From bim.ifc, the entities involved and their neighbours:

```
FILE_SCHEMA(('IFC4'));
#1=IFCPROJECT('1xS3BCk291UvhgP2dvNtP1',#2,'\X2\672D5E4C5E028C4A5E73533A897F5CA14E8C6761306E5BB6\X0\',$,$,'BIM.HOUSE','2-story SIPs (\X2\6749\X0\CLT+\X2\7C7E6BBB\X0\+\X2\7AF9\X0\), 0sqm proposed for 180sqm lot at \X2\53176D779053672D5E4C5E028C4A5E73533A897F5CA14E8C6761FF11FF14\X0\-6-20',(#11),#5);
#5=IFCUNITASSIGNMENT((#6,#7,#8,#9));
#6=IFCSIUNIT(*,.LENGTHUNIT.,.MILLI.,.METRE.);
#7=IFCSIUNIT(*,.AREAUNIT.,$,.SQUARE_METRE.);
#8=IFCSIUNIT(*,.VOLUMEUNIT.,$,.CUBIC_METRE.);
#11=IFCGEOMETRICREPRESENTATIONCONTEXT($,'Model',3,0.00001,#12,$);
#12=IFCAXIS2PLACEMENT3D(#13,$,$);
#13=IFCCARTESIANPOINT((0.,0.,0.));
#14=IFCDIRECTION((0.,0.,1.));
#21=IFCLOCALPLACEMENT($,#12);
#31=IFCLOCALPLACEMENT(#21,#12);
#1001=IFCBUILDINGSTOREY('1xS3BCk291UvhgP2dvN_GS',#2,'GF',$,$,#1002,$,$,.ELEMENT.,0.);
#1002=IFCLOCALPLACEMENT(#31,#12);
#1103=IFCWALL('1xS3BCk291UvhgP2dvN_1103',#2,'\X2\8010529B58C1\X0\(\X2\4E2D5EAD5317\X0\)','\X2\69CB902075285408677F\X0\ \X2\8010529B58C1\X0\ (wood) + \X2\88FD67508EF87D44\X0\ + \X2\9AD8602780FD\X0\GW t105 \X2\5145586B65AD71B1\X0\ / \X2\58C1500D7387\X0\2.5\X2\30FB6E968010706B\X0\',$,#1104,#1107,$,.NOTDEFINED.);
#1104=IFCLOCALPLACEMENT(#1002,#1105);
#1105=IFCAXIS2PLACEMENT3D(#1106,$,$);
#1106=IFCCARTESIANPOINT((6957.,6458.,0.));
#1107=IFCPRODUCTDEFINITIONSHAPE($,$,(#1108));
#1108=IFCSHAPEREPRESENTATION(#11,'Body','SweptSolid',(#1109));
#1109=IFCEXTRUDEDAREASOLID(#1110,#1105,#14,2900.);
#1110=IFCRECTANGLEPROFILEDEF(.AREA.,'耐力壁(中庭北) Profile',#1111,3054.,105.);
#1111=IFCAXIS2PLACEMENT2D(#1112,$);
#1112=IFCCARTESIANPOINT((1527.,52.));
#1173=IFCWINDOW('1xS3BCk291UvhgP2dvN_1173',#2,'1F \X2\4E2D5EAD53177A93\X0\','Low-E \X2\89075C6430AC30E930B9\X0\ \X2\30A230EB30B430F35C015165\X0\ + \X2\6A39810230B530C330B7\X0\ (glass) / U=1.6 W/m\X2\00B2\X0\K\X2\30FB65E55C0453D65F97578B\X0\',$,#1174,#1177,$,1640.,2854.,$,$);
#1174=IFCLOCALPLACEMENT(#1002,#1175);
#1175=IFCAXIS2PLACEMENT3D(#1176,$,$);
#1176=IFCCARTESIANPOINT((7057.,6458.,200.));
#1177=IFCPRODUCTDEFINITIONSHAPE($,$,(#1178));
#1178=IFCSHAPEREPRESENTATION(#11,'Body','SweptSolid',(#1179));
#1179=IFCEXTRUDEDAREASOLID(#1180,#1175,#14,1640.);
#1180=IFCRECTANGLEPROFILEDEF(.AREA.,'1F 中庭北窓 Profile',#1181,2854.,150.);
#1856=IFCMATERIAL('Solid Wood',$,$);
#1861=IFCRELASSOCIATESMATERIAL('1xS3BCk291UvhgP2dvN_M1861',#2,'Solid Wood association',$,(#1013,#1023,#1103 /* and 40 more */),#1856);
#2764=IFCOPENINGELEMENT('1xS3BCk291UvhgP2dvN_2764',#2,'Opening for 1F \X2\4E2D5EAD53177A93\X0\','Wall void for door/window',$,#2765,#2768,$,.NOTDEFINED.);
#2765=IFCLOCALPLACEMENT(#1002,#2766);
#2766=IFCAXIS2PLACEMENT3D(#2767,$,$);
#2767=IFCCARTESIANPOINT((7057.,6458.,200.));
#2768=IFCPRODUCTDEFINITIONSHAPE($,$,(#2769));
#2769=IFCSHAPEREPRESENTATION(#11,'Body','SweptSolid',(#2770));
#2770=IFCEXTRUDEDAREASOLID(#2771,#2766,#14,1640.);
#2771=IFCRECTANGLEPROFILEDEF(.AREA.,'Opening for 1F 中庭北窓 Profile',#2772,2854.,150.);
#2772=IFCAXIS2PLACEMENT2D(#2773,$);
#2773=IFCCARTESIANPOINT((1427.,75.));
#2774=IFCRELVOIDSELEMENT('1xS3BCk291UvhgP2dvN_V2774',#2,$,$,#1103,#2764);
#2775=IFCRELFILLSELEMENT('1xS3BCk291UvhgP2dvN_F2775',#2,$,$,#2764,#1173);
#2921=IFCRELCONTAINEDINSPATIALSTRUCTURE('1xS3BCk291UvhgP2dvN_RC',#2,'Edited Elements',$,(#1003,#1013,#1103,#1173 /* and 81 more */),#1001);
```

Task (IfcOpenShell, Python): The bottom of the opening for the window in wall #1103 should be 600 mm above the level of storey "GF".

```python
import numpy as np
import ifcopenshell
import ifcopenshell.api.geometry
import ifcopenshell.geom
import ifcopenshell.util.element
import ifcopenshell.util.placement
import ifcopenshell.util.shape
import ifcopenshell.util.unit

model = ifcopenshell.open("bim.ifc")
unit_scale = ifcopenshell.util.unit.calculate_unit_scale(model)

window = model.by_id(1173)
opening = window.FillsVoids[0].RelatingOpeningElement
storey = ifcopenshell.util.element.get_container(window, ifc_class="IfcBuildingStorey")
level = ifcopenshell.util.placement.get_local_placement(storey.ObjectPlacement)[2, 3]

# The opening's origin need not be at the sill, so measure its lowest point.
shape = ifcopenshell.geom.create_shape(ifcopenshell.geom.settings(), opening)
bottom = ifcopenshell.util.shape.get_shape_bottom_elevation(shape, shape.geometry) / unit_scale
dz = level + 0.6 / unit_scale - bottom

shift = np.array([0.0, 0.0, dz])
# The window is not placed relative to its opening, so move both.
for product in (opening, window):
    matrix = ifcopenshell.util.placement.get_local_placement(product.ObjectPlacement)
    matrix[:3, 3] += shift
    ifcopenshell.api.geometry.edit_object_placement(model, product=product, matrix=matrix, is_si=False)

print(f"moved by {dz * unit_scale:+.3f} m")

model.write("bim-out.ifc")
```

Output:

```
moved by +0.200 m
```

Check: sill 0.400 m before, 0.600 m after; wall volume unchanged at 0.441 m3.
